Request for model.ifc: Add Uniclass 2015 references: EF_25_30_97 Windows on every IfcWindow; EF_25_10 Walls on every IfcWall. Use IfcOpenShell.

First a look at what the model holds.

```python
import ifcopenshell

model = ifcopenshell.open("model.ifc")
print(model.schema)
print("classifications:", [c.Name for c in model.by_type("IfcClassification")])
for ifc_class in ("IfcDoor", "IfcRoof", "IfcStair", "IfcWall", "IfcWindow"):
    print(ifc_class, len(model.by_type(ifc_class)))
```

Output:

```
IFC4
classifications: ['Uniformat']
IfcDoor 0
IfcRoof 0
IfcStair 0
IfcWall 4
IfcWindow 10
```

```python
import ifcopenshell
import ifcopenshell.api.classification

model = ifcopenshell.open("model.ifc")

system = ifcopenshell.api.classification.add_classification(model, classification="Uniclass 2015")

codes = {
    "IfcWindow": ("EF_25_30_97", "Windows"),
    "IfcWall": ("EF_25_10", "Walls"),
}
for ifc_class, (code, name) in codes.items():
    products = model.by_type(ifc_class)
    ifcopenshell.api.classification.add_reference(
        model, products=products, classification=system, identification=code, name=name
    )
    print(code, len(products))

model.write("model_edited.ifc")
```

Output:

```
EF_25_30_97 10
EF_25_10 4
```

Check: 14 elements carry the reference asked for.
